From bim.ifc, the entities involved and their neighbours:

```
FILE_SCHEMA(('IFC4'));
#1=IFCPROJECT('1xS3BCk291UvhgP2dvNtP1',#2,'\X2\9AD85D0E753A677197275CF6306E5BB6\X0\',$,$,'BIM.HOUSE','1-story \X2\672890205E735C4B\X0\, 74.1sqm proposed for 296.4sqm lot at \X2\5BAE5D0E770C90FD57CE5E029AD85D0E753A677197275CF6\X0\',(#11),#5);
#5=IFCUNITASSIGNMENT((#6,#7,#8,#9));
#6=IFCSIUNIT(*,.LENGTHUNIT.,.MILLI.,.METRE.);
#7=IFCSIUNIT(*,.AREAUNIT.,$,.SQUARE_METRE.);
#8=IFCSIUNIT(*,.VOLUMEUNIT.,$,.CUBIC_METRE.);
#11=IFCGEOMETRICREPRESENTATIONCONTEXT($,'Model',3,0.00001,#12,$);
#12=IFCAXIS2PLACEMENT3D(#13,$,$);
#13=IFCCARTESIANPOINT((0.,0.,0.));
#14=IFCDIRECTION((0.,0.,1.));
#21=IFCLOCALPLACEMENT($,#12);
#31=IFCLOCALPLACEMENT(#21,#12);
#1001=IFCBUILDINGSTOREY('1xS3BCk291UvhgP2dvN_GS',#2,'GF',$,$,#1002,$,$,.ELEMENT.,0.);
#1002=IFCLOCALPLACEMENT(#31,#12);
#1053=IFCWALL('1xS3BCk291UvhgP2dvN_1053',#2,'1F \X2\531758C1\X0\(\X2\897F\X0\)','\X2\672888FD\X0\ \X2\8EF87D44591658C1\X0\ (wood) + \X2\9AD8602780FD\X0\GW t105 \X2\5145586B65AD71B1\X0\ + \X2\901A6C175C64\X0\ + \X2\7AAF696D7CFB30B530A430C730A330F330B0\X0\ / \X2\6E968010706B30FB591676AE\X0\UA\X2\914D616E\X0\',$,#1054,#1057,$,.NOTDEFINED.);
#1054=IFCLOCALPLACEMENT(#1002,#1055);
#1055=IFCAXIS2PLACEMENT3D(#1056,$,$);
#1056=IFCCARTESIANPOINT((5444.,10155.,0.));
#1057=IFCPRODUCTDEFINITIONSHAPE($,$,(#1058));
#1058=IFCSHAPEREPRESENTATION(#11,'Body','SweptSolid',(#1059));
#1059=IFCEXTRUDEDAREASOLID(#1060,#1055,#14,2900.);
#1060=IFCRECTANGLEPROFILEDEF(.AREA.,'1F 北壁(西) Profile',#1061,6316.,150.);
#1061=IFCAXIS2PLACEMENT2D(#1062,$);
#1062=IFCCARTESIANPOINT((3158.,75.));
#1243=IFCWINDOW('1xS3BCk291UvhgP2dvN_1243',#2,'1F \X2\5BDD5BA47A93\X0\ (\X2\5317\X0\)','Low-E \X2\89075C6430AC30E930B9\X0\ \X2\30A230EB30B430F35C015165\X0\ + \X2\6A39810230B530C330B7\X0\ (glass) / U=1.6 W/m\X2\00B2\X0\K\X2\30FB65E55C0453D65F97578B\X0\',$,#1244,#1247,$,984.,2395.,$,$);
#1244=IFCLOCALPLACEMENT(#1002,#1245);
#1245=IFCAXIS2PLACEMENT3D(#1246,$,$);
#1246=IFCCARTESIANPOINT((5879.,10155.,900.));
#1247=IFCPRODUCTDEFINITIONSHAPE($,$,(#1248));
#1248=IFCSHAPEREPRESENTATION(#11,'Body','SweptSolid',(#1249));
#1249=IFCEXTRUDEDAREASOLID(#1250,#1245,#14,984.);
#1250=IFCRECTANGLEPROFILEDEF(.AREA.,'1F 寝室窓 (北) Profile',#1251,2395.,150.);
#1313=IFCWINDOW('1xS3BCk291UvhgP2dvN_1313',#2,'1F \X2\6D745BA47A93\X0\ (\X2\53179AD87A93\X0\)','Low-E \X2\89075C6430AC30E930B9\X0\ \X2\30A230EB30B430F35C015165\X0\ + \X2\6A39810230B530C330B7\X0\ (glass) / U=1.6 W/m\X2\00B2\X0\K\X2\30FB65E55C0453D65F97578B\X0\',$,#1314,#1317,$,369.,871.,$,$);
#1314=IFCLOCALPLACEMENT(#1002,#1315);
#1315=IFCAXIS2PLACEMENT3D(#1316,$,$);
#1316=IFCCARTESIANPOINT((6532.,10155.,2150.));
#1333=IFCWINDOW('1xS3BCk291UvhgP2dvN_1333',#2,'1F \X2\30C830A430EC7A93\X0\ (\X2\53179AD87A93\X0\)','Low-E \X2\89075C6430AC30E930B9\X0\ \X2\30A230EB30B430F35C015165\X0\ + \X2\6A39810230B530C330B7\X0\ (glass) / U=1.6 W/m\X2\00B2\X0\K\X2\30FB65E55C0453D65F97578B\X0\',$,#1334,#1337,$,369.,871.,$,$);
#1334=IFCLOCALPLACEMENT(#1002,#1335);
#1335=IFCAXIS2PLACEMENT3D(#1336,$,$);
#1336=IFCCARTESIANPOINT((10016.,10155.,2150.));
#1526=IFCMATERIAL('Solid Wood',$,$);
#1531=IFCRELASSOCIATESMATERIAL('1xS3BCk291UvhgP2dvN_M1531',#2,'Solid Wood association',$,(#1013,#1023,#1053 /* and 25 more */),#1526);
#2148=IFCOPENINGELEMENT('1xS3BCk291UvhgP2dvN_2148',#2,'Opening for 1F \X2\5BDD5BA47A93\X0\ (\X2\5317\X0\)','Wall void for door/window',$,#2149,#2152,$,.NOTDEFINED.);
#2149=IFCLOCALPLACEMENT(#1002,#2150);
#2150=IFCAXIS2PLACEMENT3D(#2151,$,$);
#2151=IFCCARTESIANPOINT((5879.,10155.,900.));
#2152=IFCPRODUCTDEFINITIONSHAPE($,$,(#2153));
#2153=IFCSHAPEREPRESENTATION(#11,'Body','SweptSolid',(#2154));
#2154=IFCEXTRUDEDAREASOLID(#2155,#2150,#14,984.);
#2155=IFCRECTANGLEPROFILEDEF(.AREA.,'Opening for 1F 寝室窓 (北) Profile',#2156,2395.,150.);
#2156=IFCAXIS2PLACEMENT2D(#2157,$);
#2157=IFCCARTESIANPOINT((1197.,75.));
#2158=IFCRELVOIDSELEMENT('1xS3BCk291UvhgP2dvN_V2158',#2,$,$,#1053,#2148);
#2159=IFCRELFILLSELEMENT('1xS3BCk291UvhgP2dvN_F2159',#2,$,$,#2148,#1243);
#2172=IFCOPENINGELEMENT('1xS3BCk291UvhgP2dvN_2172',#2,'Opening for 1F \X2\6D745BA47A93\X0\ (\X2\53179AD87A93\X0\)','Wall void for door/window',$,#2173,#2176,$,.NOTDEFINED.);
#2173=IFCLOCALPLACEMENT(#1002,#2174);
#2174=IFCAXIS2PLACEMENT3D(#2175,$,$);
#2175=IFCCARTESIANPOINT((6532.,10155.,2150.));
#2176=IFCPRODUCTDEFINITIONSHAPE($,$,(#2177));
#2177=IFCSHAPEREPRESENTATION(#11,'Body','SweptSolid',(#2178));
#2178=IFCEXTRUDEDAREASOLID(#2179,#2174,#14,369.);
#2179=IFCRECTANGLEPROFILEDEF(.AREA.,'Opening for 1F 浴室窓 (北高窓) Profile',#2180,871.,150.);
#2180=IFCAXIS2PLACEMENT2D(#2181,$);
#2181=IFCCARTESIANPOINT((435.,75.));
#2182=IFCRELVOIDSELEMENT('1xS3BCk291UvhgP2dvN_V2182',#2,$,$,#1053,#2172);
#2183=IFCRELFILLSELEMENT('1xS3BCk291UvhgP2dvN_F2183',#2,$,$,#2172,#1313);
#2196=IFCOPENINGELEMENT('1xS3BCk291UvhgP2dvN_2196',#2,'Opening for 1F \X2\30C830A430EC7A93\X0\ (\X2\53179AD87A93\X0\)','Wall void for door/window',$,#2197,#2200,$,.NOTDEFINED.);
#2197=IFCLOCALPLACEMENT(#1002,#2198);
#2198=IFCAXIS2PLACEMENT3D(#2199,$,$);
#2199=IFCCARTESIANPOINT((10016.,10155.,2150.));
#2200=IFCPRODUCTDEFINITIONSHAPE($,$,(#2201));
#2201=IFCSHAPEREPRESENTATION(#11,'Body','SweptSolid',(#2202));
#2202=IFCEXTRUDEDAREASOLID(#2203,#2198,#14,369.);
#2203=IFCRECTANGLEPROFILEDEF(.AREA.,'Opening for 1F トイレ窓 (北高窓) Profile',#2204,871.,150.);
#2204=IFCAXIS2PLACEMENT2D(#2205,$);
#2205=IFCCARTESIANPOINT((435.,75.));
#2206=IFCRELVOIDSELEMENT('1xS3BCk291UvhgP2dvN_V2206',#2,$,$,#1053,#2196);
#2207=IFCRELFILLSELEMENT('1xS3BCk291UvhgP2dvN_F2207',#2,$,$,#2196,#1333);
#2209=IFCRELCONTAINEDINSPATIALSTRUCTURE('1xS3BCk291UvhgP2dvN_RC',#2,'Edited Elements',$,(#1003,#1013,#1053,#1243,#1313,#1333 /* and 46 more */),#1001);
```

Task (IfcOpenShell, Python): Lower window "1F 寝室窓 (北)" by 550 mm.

```python
import numpy as np
import ifcopenshell
import ifcopenshell.api.geometry
import ifcopenshell.util.placement
import ifcopenshell.util.unit

model = ifcopenshell.open("bim.ifc")
unit_scale = ifcopenshell.util.unit.calculate_unit_scale(model)

window = model.by_guid("1xS3BCk291UvhgP2dvN_1243")
opening = window.FillsVoids[0].RelatingOpeningElement
dz = -550.0

shift = np.array([0.0, 0.0, dz])
# The window is not placed relative to its opening, so move both.
for product in (opening, window):
    matrix = ifcopenshell.util.placement.get_local_placement(product.ObjectPlacement)
    matrix[:3, 3] += shift
    ifcopenshell.api.geometry.edit_object_placement(model, product=product, matrix=matrix, is_si=False)

print(f"moved by {dz * unit_scale:+.3f} m")

model.write("bim-out.ifc")
```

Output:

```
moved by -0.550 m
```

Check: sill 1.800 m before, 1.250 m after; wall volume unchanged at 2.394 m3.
